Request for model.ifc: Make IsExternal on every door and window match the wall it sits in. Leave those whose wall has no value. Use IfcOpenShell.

First a look at what the model holds.

```python
import ifcopenshell
import ifcopenshell.util.element

model = ifcopenshell.open("model.ifc")
print(model.schema)
seen = {}
for e in model.by_type("IfcDoor") + model.by_type("IfcWindow"):
    if not e.FillsVoids:
        continue
    host = e.FillsVoids[0].RelatingOpeningElement.VoidsElements[0].RelatingBuildingElement
    own = ifcopenshell.util.element.get_pset(e, f"Pset_{e.is_a()[3:].removesuffix('StandardCase')}Common", "IsExternal")
    wall = ifcopenshell.util.element.get_pset(host, "Pset_WallCommon", "IsExternal")
    seen[e.is_a(), own, wall] = seen.get((e.is_a(), own, wall), 0) + 1
for (cls, own, wall), count in sorted(seen.items(), key=str):
    print(count, cls, "IsExternal:", own, "| host wall:", wall)
```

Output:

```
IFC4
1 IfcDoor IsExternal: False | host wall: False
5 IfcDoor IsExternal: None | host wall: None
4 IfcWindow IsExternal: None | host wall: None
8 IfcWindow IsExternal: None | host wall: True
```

```python
import ifcopenshell
import ifcopenshell.api.pset
import ifcopenshell.util.element

model = ifcopenshell.open("model.ifc")

count = 0
for ifc_class, pset_name in (("IfcDoor", "Pset_DoorCommon"), ("IfcWindow", "Pset_WindowCommon")):
    for e in model.by_type(ifc_class):
        if not e.FillsVoids:
            continue
        host = e.FillsVoids[0].RelatingOpeningElement.VoidsElements[0].RelatingBuildingElement
        external = ifcopenshell.util.element.get_pset(host, "Pset_WallCommon", "IsExternal")
        if external is None or ifcopenshell.util.element.get_pset(e, pset_name, "IsExternal") == external:
            continue
        pset = ifcopenshell.api.pset.add_pset(model, product=e, name=pset_name)
        ifcopenshell.api.pset.edit_pset(model, pset=pset, properties={"IsExternal": external})
        count += 1

print(count, "updated")

model.write("model_rev.ifc")
```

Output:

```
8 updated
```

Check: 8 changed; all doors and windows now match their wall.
